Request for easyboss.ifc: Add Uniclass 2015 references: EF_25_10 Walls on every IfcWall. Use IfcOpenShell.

First a look at what the model holds.

```python
import ifcopenshell

model = ifcopenshell.open("easyboss.ifc")
print(model.schema)
print("classifications:", [c.Name for c in model.by_type("IfcClassification")])
for ifc_class in ("IfcDoor", "IfcRoof", "IfcStair", "IfcWall", "IfcWindow"):
    print(ifc_class, len(model.by_type(ifc_class)))
```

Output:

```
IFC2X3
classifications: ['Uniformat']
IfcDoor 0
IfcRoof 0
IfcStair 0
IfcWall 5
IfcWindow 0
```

```python
import ifcopenshell
import ifcopenshell.api.classification

model = ifcopenshell.open("easyboss.ifc")

# IFC2X3 requires Source and Edition and has no link from the project to the system.
system = model.create_entity("IfcClassification", Source="NBS", Edition="2015", Name="Uniclass 2015")

codes = {
    "IfcWall": ("EF_25_10", "Walls"),
}
for ifc_class, (code, name) in codes.items():
    products = model.by_type(ifc_class)
    ifcopenshell.api.classification.add_reference(
        model, products=products, classification=system, identification=code, name=name
    )
    print(code, len(products))

model.write("easyboss-out.ifc")
```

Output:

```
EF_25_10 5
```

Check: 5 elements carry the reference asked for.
